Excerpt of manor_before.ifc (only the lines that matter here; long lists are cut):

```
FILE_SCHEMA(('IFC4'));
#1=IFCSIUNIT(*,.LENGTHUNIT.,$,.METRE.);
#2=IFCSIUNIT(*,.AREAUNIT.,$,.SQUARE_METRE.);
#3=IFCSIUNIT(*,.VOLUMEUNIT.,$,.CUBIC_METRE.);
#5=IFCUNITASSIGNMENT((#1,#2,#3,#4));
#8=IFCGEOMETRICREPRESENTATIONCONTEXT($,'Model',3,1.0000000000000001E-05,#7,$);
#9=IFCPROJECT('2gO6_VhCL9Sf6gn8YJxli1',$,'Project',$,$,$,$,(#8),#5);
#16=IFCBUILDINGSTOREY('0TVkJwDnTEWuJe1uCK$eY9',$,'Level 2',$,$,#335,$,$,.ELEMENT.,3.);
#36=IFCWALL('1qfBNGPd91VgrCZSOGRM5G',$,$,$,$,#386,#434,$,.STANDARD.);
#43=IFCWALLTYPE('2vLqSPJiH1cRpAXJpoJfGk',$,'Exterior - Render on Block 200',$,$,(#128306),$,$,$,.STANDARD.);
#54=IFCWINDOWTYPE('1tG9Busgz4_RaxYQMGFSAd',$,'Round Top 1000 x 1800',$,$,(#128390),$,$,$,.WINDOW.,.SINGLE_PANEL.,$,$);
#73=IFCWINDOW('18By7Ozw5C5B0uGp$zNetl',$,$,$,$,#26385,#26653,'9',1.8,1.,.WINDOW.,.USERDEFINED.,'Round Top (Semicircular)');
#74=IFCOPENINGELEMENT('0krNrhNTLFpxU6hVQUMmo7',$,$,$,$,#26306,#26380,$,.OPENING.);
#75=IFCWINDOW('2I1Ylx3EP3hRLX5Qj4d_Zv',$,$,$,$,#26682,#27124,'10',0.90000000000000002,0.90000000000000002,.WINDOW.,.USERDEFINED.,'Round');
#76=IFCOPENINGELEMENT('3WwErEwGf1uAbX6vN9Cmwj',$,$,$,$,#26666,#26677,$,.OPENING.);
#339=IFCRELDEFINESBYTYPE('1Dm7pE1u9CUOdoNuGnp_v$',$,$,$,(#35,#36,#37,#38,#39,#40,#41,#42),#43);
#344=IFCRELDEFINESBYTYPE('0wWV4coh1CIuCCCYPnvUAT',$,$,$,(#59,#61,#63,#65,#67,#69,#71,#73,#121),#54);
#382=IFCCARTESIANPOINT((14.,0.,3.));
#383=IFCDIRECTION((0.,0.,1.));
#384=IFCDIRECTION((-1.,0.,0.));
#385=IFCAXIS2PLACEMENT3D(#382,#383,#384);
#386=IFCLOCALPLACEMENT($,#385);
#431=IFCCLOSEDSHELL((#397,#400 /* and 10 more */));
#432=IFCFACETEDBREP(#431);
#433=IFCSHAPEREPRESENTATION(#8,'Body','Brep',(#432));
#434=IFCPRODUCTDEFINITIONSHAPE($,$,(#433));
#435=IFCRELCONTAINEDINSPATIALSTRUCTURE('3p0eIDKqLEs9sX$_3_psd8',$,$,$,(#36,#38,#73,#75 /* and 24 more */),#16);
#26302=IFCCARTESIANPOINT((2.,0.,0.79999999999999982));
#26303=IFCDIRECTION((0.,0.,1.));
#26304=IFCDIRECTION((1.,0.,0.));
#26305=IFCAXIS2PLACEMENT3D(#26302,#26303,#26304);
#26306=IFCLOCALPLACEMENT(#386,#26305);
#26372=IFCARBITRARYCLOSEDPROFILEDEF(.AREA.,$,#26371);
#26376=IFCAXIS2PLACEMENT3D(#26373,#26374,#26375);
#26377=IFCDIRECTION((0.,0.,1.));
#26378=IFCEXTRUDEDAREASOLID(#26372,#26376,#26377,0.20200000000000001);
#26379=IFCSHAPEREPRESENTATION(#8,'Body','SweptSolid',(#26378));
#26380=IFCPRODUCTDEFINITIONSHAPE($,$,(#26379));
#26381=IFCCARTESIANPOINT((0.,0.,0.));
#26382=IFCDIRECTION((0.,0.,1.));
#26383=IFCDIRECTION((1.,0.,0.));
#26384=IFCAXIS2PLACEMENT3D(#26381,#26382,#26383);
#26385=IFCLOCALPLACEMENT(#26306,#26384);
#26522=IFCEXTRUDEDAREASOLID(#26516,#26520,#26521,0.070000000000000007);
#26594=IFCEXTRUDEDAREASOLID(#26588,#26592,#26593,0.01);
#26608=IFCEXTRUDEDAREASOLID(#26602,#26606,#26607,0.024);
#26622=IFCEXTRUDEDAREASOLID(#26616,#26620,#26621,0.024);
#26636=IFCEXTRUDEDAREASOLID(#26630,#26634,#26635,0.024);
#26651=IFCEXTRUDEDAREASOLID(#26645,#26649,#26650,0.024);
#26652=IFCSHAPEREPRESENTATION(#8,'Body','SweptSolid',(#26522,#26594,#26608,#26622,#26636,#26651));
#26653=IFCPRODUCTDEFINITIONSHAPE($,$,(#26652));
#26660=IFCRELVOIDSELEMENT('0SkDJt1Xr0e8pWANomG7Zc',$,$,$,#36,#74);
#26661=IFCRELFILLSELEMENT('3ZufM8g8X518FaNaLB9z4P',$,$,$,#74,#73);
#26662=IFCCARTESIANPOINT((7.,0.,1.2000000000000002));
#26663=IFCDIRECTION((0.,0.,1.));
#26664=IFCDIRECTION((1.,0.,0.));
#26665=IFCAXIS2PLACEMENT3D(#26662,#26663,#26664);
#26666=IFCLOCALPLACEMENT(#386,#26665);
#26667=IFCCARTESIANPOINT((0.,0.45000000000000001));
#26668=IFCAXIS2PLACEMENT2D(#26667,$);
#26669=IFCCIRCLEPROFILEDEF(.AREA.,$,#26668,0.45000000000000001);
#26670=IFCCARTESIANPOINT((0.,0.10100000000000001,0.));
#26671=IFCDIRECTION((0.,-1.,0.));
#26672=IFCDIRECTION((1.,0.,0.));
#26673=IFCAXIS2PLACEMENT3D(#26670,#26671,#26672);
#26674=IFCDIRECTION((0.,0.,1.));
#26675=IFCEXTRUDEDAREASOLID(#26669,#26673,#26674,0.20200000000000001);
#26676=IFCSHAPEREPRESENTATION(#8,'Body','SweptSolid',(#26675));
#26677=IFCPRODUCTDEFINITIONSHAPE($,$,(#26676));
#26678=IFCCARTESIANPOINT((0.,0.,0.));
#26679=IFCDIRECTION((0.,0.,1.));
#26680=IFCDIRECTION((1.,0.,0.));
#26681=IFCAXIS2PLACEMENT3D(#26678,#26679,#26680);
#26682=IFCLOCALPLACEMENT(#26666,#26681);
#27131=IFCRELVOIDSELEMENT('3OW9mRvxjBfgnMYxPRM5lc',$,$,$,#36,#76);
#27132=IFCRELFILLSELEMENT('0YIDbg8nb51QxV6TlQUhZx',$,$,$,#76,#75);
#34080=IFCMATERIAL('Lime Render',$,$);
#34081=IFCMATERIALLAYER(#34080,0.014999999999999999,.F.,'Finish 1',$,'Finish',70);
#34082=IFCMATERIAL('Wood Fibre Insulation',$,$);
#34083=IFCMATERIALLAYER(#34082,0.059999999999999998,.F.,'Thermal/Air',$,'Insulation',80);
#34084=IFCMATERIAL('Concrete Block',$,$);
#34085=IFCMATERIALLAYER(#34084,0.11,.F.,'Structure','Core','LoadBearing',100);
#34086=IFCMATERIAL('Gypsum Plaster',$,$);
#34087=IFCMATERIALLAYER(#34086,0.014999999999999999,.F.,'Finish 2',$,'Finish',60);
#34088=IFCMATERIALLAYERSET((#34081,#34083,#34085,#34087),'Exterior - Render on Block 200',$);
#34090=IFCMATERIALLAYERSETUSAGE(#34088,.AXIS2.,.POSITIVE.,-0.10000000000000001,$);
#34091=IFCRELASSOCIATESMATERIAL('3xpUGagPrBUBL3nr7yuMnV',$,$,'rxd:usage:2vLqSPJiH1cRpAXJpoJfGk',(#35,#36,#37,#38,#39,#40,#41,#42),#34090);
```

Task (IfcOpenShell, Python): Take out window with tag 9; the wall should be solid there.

```python
import ifcopenshell
import ifcopenshell.api.feature
import ifcopenshell.api.root
import ifcopenshell.geom
import ifcopenshell.util.shape

model = ifcopenshell.open("manor_before.ifc")
settings = ifcopenshell.geom.settings()


def volume(element):
    """Net volume in cubic metres, openings subtracted."""
    shape = ifcopenshell.geom.create_shape(settings, element)
    return ifcopenshell.util.shape.get_volume(shape.geometry)


window = model.by_guid("18By7Ozw5C5B0uGp$zNetl")
opening = window.FillsVoids[0].RelatingOpeningElement
wall = opening.VoidsElements[0].RelatingBuildingElement
before = volume(wall)

ifcopenshell.api.root.remove_product(model, product=window)
ifcopenshell.api.feature.remove_feature(model, feature=opening)

after = volume(wall)

print(f"wall volume {before:.3f} -> {after:.3f} m3")

model.write("manor_before_edited.ifc")
```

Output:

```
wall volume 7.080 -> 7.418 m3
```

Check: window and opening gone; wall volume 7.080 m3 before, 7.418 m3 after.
